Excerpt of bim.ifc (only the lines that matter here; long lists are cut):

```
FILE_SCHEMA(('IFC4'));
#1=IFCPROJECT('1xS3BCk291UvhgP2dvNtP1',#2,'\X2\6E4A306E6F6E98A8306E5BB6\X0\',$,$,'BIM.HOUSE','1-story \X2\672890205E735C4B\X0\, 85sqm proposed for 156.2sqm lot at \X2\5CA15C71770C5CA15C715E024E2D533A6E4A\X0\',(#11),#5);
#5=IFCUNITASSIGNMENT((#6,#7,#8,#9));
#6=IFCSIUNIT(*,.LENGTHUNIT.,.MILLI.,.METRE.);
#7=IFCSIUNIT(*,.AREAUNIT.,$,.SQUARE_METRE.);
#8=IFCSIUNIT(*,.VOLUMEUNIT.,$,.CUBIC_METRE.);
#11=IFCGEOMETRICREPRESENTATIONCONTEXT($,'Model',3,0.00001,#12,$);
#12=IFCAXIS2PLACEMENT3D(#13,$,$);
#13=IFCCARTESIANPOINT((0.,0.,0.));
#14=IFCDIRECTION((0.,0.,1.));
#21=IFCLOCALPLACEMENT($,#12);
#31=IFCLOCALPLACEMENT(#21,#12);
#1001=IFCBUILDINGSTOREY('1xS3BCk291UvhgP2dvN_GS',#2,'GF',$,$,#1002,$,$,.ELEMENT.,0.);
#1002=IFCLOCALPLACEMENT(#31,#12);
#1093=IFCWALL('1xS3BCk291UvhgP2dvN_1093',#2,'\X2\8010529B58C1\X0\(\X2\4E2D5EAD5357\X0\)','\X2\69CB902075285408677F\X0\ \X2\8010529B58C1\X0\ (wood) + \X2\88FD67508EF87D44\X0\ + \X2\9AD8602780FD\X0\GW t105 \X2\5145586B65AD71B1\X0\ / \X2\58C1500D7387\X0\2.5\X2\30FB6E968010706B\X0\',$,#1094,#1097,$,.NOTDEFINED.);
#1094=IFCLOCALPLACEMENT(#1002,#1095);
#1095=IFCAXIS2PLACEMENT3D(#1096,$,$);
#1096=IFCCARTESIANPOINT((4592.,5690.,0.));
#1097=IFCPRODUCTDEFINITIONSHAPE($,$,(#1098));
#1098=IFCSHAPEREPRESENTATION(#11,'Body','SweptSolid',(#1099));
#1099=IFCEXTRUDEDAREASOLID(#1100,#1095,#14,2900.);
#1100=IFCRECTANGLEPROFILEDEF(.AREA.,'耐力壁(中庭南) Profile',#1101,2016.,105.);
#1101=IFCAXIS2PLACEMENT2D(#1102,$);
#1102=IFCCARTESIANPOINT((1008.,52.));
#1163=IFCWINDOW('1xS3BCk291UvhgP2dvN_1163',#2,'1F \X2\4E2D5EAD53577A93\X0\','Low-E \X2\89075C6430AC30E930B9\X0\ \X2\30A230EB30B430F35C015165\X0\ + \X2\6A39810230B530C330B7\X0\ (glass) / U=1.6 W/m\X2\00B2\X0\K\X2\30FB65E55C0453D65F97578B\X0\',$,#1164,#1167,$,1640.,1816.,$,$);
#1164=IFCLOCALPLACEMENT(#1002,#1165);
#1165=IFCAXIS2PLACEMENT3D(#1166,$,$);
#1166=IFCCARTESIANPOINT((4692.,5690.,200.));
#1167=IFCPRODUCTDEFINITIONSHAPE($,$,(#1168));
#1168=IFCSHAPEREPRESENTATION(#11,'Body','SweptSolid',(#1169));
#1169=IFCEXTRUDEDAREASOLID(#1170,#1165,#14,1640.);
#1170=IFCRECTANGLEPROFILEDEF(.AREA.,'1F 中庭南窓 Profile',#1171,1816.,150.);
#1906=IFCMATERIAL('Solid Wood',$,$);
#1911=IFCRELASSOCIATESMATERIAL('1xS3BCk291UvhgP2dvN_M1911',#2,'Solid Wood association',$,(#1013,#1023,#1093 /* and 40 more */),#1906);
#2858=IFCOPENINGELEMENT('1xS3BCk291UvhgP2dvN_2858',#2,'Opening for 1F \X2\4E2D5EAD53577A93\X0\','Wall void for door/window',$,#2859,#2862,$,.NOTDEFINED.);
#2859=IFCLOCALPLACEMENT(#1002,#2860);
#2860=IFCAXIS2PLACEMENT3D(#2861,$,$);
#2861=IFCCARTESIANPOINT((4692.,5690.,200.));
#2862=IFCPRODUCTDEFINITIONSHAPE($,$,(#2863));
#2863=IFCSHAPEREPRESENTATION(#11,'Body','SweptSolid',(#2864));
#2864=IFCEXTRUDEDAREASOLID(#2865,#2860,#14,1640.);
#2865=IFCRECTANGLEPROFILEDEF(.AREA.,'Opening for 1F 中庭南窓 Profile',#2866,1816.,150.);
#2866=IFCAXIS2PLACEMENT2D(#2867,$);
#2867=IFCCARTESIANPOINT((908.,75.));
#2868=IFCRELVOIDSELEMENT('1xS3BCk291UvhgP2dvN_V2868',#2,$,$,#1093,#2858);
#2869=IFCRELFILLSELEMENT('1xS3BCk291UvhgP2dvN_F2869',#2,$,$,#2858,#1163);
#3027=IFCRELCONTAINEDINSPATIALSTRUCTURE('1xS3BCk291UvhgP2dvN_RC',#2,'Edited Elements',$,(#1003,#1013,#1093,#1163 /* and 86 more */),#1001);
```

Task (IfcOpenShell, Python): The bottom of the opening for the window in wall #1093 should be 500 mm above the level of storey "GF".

```python
import numpy as np
import ifcopenshell
import ifcopenshell.api.geometry
import ifcopenshell.geom
import ifcopenshell.util.element
import ifcopenshell.util.placement
import ifcopenshell.util.shape
import ifcopenshell.util.unit

model = ifcopenshell.open("bim.ifc")
unit_scale = ifcopenshell.util.unit.calculate_unit_scale(model)

window = model.by_guid("1xS3BCk291UvhgP2dvN_1163")
opening = window.FillsVoids[0].RelatingOpeningElement
storey = ifcopenshell.util.element.get_container(window, ifc_class="IfcBuildingStorey")
level = ifcopenshell.util.placement.get_local_placement(storey.ObjectPlacement)[2, 3]

# The opening's origin need not be at the sill, so measure its lowest point.
shape = ifcopenshell.geom.create_shape(ifcopenshell.geom.settings(), opening)
bottom = ifcopenshell.util.shape.get_shape_bottom_elevation(shape, shape.geometry) / unit_scale
dz = level + 0.5 / unit_scale - bottom

shift = np.array([0.0, 0.0, dz])
# The window is not placed relative to its opening, so move both.
for product in (opening, window):
    matrix = ifcopenshell.util.placement.get_local_placement(product.ObjectPlacement)
    matrix[:3, 3] += shift
    ifcopenshell.api.geometry.edit_object_placement(model, product=product, matrix=matrix, is_si=False)

print(f"moved by {dz * unit_scale:+.3f} m")

model.write("bim_edited.ifc")
```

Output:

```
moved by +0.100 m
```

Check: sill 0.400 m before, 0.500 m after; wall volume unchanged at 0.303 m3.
